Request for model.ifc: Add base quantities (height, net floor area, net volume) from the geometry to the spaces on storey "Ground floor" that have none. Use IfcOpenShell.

First a look at what the model holds.

```python
import ifcopenshell
import ifcopenshell.util.element
import ifcopenshell.util.unit

model = ifcopenshell.open("model.ifc")
print(model.schema)
for unit_type in ("LENGTHUNIT", "AREAUNIT", "VOLUMEUNIT"):
    print(unit_type, ifcopenshell.util.unit.calculate_unit_scale(model, unit_type))
storey = next(s for s in model.by_type("IfcBuildingStorey") if s.Name == "Ground floor")
spaces = [e for e in ifcopenshell.util.element.get_decomposition(storey) if e.is_a("IfcSpace")]
for e in sorted(spaces, key=lambda e: e.id()):
    print(e.id(), e.is_a(), e.Name, list(ifcopenshell.util.element.get_psets(e, qtos_only=True)), sep=" | ")
```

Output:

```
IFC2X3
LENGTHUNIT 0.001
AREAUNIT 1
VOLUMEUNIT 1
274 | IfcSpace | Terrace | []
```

```python
import ifcopenshell
import ifcopenshell.api.pset
import ifcopenshell.geom
import ifcopenshell.util.element
import ifcopenshell.util.shape
import ifcopenshell.util.unit

model = ifcopenshell.open("model.ifc")
unit_scale = ifcopenshell.util.unit.calculate_unit_scale(model)
area_scale = ifcopenshell.util.unit.calculate_unit_scale(model, "AREAUNIT")
volume_scale = ifcopenshell.util.unit.calculate_unit_scale(model, "VOLUMEUNIT")
settings = ifcopenshell.geom.settings()

storey = next(s for s in model.by_type("IfcBuildingStorey") if s.Name == "Ground floor")
spaces = [e for e in ifcopenshell.util.element.get_decomposition(storey) if e.is_a("IfcSpace")]

for e in sorted(spaces, key=lambda e: e.id()):
    if ifcopenshell.util.element.get_psets(e, qtos_only=True, should_inherit=False):
        continue
    # Geometry comes back in metres, in the element's own axes.
    shape = ifcopenshell.geom.create_shape(settings, e)
    values = {
        "Height": ifcopenshell.util.shape.get_z(shape.geometry) / unit_scale,
        "NetFloorArea": ifcopenshell.util.shape.get_footprint_area(shape.geometry) / area_scale,
        "NetVolume": ifcopenshell.util.shape.get_volume(shape.geometry) / volume_scale,
    }
    qto = ifcopenshell.api.pset.add_qto(model, product=e, name="BaseQuantities")
    ifcopenshell.api.pset.edit_qto(model, qto=qto, properties=values)
    print(e.id(), {k: round(v, 3) for k, v in values.items()})

model.write("model_rev.ifc")
```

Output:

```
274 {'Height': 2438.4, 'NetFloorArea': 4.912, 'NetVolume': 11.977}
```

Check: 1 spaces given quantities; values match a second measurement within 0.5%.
